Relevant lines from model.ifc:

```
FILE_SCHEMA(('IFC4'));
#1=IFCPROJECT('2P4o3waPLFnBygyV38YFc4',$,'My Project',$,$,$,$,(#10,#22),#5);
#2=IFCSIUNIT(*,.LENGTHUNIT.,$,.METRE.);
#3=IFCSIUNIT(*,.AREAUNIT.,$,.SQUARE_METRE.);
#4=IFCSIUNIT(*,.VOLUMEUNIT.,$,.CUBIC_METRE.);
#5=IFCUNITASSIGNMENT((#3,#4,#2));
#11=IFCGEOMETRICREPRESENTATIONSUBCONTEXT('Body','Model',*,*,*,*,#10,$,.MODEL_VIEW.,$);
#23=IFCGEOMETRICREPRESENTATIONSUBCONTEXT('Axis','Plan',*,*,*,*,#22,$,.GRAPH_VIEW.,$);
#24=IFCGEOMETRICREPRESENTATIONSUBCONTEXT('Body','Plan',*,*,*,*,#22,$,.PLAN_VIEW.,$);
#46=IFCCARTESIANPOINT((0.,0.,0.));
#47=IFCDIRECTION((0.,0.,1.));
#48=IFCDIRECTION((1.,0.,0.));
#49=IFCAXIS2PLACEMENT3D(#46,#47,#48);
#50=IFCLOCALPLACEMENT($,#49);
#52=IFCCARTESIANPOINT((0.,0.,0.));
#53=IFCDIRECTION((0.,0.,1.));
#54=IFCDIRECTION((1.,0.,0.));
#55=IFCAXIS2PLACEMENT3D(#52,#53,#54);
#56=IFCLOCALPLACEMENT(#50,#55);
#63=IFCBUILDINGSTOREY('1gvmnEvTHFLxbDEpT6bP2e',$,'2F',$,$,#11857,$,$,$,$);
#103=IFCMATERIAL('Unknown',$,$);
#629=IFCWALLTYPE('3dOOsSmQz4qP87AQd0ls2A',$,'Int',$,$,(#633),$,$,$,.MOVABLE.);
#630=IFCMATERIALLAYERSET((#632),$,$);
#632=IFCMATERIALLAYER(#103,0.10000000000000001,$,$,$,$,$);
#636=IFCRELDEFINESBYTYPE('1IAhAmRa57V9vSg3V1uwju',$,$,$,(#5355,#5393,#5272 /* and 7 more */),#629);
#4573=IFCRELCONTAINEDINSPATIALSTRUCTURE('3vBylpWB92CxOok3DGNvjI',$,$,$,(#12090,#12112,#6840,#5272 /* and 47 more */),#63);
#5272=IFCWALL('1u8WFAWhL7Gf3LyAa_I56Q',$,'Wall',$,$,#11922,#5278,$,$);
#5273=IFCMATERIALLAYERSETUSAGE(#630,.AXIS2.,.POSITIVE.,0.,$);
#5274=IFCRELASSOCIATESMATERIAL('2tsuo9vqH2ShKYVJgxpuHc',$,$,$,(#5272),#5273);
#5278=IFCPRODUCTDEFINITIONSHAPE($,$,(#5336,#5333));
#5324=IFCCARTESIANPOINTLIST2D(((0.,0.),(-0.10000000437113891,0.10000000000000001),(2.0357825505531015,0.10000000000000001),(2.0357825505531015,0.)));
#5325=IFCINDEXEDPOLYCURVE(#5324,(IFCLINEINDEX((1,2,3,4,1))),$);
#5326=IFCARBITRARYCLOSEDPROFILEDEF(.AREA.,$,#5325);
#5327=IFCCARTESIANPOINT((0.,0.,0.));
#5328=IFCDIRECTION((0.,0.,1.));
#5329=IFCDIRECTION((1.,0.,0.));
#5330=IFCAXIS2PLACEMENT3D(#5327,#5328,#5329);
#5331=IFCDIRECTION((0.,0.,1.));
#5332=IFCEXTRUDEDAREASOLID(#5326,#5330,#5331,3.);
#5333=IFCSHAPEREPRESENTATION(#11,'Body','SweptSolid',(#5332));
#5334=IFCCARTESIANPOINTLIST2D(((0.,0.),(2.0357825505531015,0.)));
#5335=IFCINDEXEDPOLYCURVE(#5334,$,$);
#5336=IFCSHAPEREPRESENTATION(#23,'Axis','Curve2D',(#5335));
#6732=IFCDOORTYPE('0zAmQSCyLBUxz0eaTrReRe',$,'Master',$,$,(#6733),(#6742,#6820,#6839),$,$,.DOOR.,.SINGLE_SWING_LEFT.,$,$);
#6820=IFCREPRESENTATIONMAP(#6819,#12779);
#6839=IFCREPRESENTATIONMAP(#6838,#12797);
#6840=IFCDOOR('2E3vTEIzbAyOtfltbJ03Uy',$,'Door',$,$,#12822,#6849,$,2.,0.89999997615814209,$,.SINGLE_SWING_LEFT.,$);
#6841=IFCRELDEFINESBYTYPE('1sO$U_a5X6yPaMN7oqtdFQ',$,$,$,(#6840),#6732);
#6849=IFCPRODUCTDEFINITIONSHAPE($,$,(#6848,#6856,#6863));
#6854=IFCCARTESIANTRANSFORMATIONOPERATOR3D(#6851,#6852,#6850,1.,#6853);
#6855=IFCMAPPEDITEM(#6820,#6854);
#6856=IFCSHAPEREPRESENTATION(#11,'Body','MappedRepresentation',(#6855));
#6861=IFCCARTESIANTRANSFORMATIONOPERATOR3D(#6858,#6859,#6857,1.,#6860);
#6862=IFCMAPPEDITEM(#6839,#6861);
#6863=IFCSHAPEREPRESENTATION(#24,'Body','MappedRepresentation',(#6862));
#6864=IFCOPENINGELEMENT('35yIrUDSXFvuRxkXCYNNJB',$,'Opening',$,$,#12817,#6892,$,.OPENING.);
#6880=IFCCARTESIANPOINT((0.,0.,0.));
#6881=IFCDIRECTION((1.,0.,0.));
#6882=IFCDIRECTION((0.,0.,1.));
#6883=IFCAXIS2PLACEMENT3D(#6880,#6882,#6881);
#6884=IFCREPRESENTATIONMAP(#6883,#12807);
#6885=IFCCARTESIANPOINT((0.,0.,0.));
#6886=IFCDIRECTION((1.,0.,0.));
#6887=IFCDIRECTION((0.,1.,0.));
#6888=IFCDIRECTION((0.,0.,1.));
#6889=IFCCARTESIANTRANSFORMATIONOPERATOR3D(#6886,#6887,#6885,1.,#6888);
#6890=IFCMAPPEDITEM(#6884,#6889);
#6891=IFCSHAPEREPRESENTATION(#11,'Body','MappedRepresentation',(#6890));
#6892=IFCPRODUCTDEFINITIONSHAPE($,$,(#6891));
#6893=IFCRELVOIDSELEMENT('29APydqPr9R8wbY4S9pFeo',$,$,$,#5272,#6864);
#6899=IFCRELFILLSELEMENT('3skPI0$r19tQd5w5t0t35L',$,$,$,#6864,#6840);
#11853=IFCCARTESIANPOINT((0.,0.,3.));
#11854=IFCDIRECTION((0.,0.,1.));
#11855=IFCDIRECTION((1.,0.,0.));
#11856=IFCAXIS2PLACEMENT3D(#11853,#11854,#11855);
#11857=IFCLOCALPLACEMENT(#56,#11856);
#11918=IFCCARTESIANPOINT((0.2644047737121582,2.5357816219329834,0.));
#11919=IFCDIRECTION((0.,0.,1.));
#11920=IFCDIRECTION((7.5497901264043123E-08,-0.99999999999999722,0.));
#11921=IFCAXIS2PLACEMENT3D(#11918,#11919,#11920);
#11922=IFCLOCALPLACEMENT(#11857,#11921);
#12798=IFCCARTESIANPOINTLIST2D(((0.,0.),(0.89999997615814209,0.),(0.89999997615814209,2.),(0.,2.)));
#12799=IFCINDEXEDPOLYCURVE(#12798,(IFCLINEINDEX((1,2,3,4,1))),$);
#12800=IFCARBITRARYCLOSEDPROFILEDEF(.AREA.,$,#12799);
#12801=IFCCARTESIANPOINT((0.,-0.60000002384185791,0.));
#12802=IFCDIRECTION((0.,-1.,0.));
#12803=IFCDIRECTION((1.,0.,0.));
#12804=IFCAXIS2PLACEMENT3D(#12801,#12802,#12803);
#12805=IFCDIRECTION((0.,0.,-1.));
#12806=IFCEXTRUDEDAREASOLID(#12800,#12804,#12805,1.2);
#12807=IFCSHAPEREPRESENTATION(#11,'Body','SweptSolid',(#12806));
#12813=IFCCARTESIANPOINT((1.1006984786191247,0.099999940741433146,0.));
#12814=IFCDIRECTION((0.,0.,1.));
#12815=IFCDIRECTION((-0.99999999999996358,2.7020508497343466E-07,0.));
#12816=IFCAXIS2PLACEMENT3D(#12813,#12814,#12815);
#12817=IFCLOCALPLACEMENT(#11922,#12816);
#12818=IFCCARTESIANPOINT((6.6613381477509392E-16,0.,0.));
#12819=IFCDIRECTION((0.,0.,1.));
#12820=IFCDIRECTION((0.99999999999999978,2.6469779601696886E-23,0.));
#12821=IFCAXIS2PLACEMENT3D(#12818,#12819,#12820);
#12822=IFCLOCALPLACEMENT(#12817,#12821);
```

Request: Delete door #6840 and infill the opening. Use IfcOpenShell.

```python
import ifcopenshell
import ifcopenshell.api.feature
import ifcopenshell.api.root
import ifcopenshell.geom
import ifcopenshell.util.shape

model = ifcopenshell.open("model.ifc")
settings = ifcopenshell.geom.settings()


def volume(element):
    """Net volume in cubic metres, openings subtracted."""
    shape = ifcopenshell.geom.create_shape(settings, element)
    return ifcopenshell.util.shape.get_volume(shape.geometry)


door = model.by_id(6840)
opening = door.FillsVoids[0].RelatingOpeningElement
wall = opening.VoidsElements[0].RelatingBuildingElement
before = volume(wall)

ifcopenshell.api.root.remove_product(model, product=door)
ifcopenshell.api.feature.remove_feature(model, feature=opening)

after = volume(wall)

print(f"wall volume {before:.3f} -> {after:.3f} m3")

model.write("model_updated.ifc")
```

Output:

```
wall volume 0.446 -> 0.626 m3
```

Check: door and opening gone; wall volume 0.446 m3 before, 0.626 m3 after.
